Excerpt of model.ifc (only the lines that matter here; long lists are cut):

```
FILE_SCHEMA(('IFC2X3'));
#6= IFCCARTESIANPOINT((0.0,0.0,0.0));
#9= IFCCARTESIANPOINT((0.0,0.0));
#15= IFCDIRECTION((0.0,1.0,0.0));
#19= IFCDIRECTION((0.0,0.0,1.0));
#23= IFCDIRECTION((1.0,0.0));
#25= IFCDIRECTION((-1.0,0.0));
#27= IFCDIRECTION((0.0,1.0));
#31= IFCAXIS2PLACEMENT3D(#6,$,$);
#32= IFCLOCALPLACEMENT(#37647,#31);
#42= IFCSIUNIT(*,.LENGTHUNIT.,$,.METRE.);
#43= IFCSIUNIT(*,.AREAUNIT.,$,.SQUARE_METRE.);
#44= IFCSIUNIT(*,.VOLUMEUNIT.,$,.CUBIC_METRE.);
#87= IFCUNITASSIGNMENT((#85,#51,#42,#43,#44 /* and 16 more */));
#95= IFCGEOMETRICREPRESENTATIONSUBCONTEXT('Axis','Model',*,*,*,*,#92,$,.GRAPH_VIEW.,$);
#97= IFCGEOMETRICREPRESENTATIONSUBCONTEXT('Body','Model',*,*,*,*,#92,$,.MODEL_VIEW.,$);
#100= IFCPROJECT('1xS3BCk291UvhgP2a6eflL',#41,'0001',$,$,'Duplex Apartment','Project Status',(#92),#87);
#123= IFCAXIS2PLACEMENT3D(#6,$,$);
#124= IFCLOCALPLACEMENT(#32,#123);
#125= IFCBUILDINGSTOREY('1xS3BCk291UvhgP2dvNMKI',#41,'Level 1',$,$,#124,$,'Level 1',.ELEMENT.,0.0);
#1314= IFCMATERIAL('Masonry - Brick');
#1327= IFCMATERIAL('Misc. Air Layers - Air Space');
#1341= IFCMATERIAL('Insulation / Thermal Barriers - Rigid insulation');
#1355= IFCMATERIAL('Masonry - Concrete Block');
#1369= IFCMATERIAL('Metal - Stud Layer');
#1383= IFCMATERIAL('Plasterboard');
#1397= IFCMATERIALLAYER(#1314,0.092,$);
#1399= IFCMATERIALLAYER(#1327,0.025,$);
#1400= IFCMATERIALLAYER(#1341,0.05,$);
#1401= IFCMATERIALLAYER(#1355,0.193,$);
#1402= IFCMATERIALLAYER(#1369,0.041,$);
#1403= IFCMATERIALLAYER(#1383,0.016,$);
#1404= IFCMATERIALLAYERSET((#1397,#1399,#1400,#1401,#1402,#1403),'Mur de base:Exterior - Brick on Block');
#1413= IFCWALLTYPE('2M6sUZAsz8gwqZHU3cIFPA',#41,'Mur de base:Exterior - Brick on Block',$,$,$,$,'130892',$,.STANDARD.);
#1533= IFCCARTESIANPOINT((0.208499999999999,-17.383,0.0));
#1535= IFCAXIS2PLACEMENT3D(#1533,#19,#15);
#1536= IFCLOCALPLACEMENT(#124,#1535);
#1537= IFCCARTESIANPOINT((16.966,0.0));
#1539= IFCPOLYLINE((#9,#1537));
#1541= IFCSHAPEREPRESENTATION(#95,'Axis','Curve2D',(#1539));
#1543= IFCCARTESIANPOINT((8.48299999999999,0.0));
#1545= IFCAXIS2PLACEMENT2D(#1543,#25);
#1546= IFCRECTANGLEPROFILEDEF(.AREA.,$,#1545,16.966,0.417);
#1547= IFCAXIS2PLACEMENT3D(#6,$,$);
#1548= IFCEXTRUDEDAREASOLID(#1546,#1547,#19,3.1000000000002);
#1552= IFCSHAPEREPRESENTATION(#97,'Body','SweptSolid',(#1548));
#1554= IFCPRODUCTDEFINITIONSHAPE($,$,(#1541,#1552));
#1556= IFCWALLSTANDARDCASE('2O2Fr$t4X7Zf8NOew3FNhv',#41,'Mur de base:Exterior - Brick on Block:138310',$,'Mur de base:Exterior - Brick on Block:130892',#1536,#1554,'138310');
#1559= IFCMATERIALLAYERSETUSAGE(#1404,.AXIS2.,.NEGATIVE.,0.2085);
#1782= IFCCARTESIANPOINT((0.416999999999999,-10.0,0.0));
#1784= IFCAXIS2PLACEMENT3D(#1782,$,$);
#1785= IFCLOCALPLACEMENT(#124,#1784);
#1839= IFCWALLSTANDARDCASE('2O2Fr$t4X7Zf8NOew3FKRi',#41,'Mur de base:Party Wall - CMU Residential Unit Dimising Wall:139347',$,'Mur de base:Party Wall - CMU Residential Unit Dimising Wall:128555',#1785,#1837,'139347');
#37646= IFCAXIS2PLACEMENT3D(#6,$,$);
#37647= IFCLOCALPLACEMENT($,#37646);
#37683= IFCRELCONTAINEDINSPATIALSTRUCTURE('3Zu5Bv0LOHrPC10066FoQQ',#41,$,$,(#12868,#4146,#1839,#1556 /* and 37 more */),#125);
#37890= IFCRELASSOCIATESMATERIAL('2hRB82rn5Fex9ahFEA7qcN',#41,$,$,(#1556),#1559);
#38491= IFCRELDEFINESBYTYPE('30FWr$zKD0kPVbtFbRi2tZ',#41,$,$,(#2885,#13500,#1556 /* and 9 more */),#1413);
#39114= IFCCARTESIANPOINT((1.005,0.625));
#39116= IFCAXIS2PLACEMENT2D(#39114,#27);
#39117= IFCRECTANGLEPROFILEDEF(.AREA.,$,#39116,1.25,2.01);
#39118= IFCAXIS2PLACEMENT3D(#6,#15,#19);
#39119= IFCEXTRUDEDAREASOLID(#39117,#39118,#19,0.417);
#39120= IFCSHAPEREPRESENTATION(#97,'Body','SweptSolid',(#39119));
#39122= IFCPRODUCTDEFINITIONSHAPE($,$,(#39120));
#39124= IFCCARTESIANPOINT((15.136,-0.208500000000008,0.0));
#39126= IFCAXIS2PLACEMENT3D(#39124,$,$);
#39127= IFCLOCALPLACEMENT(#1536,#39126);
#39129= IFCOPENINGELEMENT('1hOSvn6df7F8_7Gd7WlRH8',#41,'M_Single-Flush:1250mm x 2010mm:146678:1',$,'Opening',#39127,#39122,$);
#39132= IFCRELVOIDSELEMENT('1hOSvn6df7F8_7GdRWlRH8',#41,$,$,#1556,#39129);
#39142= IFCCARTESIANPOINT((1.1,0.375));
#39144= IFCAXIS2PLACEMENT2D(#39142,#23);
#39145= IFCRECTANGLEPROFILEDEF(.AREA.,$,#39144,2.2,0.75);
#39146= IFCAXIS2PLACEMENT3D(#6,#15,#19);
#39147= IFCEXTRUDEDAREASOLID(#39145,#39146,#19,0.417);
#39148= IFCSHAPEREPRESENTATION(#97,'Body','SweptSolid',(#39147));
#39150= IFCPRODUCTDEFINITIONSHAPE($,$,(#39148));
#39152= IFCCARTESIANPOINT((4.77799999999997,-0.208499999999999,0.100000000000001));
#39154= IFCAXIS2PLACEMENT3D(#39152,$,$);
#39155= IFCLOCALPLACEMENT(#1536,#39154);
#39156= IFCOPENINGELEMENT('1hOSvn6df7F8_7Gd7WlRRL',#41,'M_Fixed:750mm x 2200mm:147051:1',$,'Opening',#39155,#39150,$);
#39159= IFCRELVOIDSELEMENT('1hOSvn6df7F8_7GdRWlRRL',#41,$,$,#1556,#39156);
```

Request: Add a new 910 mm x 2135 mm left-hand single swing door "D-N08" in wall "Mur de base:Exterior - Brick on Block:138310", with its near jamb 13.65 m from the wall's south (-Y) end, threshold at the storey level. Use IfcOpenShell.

```python
import numpy as np
import ifcopenshell
import ifcopenshell.api.feature
import ifcopenshell.api.geometry
import ifcopenshell.api.root
import ifcopenshell.api.spatial
import ifcopenshell.api.type
import ifcopenshell.geom
import ifcopenshell.util.element
import ifcopenshell.util.placement
import ifcopenshell.util.representation
import ifcopenshell.util.shape
import ifcopenshell.util.unit

model = ifcopenshell.open("model.ifc")
unit_scale = ifcopenshell.util.unit.calculate_unit_scale(model)
settings = ifcopenshell.geom.settings()


def volume(element):
    """Net volume in cubic metres, openings subtracted."""
    shape = ifcopenshell.geom.create_shape(settings, element)
    return ifcopenshell.util.shape.get_volume(shape.geometry)


wall = model.by_guid("2O2Fr$t4X7Zf8NOew3FNhv")
storey = ifcopenshell.util.element.get_container(wall, ifc_class="IfcBuildingStorey")
context = ifcopenshell.util.representation.get_context(model, "Model", "Body", "MODEL_VIEW")
before = volume(wall)

width, height, from_end, sill = 0.91, 2.135, 13.65, 0.0  # metres

# The wall runs along its own X axis, and the end named is its -X end.
wall_shape = ifcopenshell.geom.create_shape(settings, wall)
x, y, z = ifcopenshell.util.shape.get_vertices(wall_shape.geometry).T
start = x.min() + from_end
face, thickness = float(y.min()), float(y.max() - y.min())
wall_matrix = ifcopenshell.util.placement.get_local_placement(wall.ObjectPlacement)
level = ifcopenshell.util.placement.get_local_placement(storey.ObjectPlacement)[2, 3]


def in_wall(x, y):
    """Placement at x, y metres in the wall's axes, at sill height."""
    matrix = wall_matrix.copy()
    matrix[:, 3] = wall_matrix @ np.array([x / unit_scale, y / unit_scale, 0.0, 1.0])
    matrix[2, 3] = level + sill / unit_scale
    return matrix


# Opening: a box that overshoots both wall faces by 50 mm.
opening = ifcopenshell.api.root.create_entity(model, ifc_class="IfcOpeningElement")
box = ifcopenshell.api.geometry.add_wall_representation(
    model, context=context, length=width, height=height, thickness=thickness + 0.1
)
ifcopenshell.api.geometry.assign_representation(model, product=opening, representation=box)
ifcopenshell.api.geometry.edit_object_placement(model, product=opening, matrix=in_wall(start, face - 0.05), is_si=False)
ifcopenshell.api.feature.add_feature(model, feature=opening, element=wall)

door = ifcopenshell.api.root.create_entity(model, ifc_class="IfcDoor", name="D-N08")
door.OverallWidth, door.OverallHeight = width / unit_scale, height / unit_scale
body = ifcopenshell.api.geometry.add_door_representation(
    model,
    context=context,
    overall_width=door.OverallWidth,
    overall_height=door.OverallHeight,
    operation_type="SINGLE_SWING_LEFT",
    lining_properties={"LiningDepth": thickness / unit_scale, "ThresholdDepth": thickness / unit_scale},
)
ifcopenshell.api.geometry.assign_representation(model, product=door, representation=body)
ifcopenshell.api.spatial.assign_container(model, products=[door], relating_structure=storey)
fills = ifcopenshell.api.feature.add_filling(model, opening=opening, element=door)
fills.OwnerHistory = door.OwnerHistory  # required in IFC2X3

# IFC2X3 keeps the operation on the door style.
style = ifcopenshell.api.root.create_entity(model, ifc_class="IfcDoorStyle", name="D-N08")
style.OperationType, style.ConstructionType = "SINGLE_SWING_LEFT", "NOTDEFINED"
style.ParameterTakesPrecedence = style.Sizeable = False
ifcopenshell.api.type.assign_type(model, related_objects=[door], relating_type=style)

# The lining spans the wall, so the door starts at the wall face.
ifcopenshell.api.geometry.edit_object_placement(model, product=door, matrix=in_wall(start, face), is_si=False)

after = volume(wall)

print(f"wall volume {before:.3f} -> {after:.3f} m3")

model.write("model_v2.ifc")
```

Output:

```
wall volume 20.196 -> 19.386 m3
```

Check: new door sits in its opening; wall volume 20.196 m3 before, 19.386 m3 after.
